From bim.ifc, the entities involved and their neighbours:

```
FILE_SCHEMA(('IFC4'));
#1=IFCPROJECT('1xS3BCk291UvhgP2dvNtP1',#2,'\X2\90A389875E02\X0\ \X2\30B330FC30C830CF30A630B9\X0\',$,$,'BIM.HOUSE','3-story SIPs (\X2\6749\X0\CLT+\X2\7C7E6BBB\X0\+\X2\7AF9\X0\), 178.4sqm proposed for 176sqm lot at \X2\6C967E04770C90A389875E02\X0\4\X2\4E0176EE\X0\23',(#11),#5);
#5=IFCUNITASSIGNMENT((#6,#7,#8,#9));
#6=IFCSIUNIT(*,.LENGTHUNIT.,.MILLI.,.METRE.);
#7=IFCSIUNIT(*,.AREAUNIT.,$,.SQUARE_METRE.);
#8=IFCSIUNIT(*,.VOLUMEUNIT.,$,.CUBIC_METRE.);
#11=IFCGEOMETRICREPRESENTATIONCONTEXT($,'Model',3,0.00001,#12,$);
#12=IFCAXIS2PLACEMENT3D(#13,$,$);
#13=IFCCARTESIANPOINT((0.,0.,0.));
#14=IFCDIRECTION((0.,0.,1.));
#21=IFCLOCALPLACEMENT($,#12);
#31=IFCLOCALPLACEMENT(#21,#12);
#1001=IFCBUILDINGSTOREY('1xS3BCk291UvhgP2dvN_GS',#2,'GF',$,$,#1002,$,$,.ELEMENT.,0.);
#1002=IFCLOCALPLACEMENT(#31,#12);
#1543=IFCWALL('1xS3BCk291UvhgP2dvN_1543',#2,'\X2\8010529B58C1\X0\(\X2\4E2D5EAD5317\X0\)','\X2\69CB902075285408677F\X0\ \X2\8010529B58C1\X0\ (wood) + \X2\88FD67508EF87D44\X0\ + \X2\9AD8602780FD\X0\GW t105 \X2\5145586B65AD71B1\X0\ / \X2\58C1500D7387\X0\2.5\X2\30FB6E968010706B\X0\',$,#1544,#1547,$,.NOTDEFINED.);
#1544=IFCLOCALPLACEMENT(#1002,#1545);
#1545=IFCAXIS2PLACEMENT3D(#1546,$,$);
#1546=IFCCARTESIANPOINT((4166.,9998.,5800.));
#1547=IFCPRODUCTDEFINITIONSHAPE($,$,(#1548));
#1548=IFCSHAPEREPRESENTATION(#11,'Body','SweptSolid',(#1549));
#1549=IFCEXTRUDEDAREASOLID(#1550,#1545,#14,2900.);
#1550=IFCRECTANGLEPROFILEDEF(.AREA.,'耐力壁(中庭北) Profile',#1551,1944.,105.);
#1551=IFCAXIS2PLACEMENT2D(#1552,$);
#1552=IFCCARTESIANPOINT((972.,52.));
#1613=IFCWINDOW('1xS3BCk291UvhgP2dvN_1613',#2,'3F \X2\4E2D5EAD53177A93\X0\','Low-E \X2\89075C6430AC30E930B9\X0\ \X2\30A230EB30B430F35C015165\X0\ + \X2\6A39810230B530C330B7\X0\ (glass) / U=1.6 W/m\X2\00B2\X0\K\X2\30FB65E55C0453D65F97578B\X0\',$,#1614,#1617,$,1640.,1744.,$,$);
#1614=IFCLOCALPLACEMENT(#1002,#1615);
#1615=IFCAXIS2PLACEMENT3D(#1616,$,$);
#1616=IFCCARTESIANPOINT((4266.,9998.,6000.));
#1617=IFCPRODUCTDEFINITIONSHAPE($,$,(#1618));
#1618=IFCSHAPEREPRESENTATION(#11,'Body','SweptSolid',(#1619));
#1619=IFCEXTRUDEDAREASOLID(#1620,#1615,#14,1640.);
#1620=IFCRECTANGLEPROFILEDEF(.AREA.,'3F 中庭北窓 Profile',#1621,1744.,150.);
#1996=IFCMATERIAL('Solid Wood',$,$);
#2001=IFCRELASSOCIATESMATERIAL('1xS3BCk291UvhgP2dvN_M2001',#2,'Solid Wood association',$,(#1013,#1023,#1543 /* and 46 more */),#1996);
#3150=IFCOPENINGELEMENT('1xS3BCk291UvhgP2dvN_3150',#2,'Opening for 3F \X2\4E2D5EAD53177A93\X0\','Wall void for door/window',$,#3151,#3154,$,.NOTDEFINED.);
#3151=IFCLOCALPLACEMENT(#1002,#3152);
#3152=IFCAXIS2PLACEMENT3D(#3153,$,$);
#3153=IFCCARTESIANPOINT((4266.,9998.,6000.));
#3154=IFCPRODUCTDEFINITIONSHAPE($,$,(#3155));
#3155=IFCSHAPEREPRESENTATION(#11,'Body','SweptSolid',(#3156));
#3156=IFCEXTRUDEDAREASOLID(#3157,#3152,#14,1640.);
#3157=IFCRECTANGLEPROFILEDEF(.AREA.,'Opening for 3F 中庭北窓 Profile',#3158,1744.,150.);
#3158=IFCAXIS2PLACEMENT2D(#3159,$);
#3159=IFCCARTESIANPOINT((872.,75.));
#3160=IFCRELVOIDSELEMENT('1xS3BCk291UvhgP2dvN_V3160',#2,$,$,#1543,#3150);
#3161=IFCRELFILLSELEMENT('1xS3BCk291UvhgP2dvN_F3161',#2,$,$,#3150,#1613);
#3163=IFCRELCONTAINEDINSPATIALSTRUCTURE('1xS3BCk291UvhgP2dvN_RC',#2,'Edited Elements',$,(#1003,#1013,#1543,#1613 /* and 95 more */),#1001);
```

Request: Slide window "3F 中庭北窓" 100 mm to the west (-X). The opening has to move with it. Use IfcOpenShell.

```python
import ifcopenshell
import ifcopenshell.api.geometry
import ifcopenshell.util.placement
import ifcopenshell.util.unit

model = ifcopenshell.open("bim.ifc")
unit_scale = ifcopenshell.util.unit.calculate_unit_scale(model)

window = model.by_guid("1xS3BCk291UvhgP2dvN_1613")
opening = window.FillsVoids[0].RelatingOpeningElement
wall = opening.VoidsElements[0].RelatingBuildingElement

wall_matrix = ifcopenshell.util.placement.get_local_placement(wall.ObjectPlacement)
shift = wall_matrix[:3, 0] * -0.1 / unit_scale
before = ifcopenshell.util.placement.get_local_placement(window.ObjectPlacement)[:3, 3].copy()

# The window is not placed relative to its opening, so move both.
for product in (opening, window):
    matrix = ifcopenshell.util.placement.get_local_placement(product.ObjectPlacement)
    matrix[:3, 3] += shift
    ifcopenshell.api.geometry.edit_object_placement(model, product=product, matrix=matrix, is_si=False)

after = ifcopenshell.util.placement.get_local_placement(window.ObjectPlacement)[:3, 3]
print("window moved by", (after - before).round(3) + 0.0)

model.write("bim_v2.ifc")
```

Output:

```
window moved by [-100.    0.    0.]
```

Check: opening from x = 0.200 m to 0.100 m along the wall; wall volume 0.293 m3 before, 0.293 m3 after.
